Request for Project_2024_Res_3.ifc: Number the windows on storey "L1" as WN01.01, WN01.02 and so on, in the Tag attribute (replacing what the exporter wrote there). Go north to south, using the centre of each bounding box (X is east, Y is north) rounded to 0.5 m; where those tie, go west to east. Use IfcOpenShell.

First a look at what the model holds.

```python
import ifcopenshell
import ifcopenshell.util.element
import ifcopenshell.util.placement

model = ifcopenshell.open("Project_2024_Res_3.ifc")
print(model.schema)
storey = next(s for s in model.by_type("IfcBuildingStorey") if s.Name == "L1")
windows = [e for e in ifcopenshell.util.element.get_decomposition(storey) if e.is_a("IfcWindow")]
for e in sorted(windows, key=lambda e: e.id()):
    origin = ifcopenshell.util.placement.get_local_placement(e.ObjectPlacement)[:3, 3]
    print(e.id(), e.Tag, e.Name, origin.round(2) + 0.0, sep=" | ")
```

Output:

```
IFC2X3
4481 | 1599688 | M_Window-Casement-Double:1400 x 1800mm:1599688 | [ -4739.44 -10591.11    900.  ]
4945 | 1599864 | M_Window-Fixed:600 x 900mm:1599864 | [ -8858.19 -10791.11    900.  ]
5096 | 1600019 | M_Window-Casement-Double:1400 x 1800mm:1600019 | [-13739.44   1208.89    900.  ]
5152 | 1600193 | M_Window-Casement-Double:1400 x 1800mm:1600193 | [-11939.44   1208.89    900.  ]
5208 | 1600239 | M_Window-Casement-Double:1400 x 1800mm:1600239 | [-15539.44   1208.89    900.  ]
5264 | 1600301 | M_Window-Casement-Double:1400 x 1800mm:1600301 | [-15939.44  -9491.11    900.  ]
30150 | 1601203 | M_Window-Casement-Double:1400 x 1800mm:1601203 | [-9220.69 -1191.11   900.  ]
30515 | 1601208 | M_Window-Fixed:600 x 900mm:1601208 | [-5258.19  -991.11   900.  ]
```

```python
import ifcopenshell
import ifcopenshell.geom
import ifcopenshell.util.element
import ifcopenshell.util.shape

model = ifcopenshell.open("Project_2024_Res_3.ifc")
settings = ifcopenshell.geom.settings()
settings.set("use-world-coords", True)


def centre(element):
    shape = ifcopenshell.geom.create_shape(settings, element)
    return ifcopenshell.util.shape.get_bbox_centroid(shape.geometry)


storey = next(s for s in model.by_type("IfcBuildingStorey") if s.Name == "L1")
windows = [e for e in ifcopenshell.util.element.get_decomposition(storey) if e.is_a("IfcWindow")]

# Insertion points can sit at a corner or the storey origin, so sort by the geometry (in metres).
centres = {e: centre(e) for e in windows}
windows.sort(key=lambda e: (-round(centres[e][1] / 0.5), centres[e][0]))

for i, e in enumerate(windows, start=1):
    number = f"WN01.{i:02d}"
    e.Tag = number
    print(e.id(), number)

model.write("Project_2024_Res_3_updated.ifc")
```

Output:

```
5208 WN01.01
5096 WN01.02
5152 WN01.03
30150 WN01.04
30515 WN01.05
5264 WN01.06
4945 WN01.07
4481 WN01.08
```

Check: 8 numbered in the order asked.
